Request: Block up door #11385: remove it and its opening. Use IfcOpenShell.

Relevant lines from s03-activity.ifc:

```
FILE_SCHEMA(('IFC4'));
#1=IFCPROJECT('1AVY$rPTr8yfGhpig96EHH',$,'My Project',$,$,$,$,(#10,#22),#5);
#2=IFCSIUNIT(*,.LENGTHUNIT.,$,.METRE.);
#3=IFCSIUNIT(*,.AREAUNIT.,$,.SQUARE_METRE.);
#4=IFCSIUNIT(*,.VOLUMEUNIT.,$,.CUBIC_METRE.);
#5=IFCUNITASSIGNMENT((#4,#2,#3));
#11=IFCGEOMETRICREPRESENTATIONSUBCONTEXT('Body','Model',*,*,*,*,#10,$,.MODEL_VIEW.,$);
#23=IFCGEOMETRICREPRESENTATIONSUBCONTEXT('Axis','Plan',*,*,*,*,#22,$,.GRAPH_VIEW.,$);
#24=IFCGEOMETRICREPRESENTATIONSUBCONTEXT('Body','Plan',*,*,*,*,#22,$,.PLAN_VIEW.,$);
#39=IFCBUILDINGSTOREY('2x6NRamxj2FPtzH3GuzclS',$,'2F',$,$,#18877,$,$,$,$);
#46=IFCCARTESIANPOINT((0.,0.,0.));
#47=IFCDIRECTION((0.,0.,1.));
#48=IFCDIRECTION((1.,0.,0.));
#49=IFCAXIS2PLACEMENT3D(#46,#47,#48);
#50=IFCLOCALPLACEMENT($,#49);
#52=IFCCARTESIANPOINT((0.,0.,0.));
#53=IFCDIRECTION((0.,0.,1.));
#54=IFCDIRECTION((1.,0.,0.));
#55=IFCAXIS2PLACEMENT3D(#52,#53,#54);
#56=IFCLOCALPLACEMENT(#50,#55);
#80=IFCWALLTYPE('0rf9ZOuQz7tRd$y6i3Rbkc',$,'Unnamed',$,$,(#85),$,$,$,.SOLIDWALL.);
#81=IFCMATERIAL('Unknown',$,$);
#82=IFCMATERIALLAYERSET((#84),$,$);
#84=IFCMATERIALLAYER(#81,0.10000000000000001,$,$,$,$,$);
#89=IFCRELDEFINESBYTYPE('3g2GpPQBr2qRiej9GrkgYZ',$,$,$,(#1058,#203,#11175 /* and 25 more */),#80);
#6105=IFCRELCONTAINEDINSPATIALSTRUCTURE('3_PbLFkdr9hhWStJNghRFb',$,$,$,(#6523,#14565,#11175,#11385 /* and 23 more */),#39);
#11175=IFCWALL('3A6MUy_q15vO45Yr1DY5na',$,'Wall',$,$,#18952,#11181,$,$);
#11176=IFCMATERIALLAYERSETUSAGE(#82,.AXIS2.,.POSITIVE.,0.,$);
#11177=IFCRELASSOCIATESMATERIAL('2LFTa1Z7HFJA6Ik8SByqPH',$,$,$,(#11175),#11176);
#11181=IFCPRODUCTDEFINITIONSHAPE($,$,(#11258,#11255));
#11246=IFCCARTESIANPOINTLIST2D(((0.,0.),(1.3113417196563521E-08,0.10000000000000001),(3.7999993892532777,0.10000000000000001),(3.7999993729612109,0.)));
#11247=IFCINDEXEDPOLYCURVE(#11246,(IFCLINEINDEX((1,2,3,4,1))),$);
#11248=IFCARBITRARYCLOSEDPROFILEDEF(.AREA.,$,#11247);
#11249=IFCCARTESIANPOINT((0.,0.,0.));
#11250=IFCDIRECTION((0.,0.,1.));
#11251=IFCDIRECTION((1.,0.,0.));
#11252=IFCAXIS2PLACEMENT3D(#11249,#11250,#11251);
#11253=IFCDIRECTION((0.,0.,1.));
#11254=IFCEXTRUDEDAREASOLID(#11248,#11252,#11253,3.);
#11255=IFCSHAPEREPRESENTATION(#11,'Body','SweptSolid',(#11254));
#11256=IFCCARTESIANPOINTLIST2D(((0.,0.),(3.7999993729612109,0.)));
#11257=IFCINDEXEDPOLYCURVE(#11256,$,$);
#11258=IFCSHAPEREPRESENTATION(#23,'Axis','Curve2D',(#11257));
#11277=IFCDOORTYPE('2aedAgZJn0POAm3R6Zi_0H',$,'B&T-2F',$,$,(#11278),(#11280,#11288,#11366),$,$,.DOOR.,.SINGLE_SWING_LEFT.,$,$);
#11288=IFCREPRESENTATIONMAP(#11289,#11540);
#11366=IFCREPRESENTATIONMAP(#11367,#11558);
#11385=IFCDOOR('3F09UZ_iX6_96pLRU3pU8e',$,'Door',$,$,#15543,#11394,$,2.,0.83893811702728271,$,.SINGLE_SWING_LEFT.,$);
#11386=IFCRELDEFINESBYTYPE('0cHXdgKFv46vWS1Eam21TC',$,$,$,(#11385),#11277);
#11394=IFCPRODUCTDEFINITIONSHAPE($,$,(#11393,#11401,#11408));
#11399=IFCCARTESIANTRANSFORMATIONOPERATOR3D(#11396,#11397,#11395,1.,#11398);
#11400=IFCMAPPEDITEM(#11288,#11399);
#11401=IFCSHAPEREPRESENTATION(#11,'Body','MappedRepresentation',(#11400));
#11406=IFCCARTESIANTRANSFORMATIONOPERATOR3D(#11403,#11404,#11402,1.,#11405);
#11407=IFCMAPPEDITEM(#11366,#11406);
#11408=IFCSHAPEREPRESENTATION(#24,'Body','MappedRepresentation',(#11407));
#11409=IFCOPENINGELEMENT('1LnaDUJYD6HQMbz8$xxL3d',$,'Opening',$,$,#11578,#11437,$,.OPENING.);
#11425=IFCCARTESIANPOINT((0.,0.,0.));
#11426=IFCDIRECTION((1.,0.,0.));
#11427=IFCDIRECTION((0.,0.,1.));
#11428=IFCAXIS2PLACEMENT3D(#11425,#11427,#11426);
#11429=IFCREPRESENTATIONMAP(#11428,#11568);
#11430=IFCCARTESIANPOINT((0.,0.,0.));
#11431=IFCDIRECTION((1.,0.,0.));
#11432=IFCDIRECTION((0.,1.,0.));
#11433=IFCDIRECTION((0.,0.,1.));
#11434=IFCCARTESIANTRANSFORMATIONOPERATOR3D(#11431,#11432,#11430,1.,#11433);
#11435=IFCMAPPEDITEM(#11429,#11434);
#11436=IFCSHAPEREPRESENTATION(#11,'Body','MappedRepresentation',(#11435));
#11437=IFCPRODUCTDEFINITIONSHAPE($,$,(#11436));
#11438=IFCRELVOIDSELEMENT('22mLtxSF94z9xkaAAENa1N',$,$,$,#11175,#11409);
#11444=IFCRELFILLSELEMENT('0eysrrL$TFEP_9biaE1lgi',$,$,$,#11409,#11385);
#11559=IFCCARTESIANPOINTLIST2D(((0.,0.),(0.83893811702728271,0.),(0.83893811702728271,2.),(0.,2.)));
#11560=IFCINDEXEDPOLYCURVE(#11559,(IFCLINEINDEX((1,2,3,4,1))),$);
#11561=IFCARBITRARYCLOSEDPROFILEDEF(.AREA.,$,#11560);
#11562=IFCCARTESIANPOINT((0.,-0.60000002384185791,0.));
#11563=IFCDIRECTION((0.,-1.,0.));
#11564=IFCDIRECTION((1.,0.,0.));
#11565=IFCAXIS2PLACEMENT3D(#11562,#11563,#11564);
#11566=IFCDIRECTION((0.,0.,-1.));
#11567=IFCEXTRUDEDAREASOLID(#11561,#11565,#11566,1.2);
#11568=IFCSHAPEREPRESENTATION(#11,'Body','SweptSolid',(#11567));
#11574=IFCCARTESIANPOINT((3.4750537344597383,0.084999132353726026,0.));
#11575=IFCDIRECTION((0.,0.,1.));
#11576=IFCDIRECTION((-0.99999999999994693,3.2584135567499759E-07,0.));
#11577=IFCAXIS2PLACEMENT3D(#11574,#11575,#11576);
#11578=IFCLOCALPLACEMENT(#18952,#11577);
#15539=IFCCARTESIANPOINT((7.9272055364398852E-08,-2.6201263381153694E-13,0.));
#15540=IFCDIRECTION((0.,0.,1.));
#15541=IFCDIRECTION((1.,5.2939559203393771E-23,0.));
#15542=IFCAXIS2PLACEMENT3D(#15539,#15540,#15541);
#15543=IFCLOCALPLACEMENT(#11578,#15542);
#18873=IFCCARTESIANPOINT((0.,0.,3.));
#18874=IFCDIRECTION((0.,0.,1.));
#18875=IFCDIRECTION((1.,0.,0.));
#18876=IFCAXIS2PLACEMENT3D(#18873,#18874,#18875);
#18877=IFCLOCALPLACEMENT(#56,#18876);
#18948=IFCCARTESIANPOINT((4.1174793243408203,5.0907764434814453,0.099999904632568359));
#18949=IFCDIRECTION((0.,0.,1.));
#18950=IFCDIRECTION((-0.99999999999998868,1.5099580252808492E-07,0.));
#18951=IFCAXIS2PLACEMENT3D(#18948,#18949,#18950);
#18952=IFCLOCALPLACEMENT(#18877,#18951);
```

```python
import ifcopenshell
import ifcopenshell.api.feature
import ifcopenshell.api.root
import ifcopenshell.geom
import ifcopenshell.util.shape

model = ifcopenshell.open("s03-activity.ifc")
settings = ifcopenshell.geom.settings()


def volume(element):
    """Net volume in cubic metres, openings subtracted."""
    shape = ifcopenshell.geom.create_shape(settings, element)
    return ifcopenshell.util.shape.get_volume(shape.geometry)


door = model.by_guid("3F09UZ_iX6_96pLRU3pU8e")
opening = door.FillsVoids[0].RelatingOpeningElement
wall = opening.VoidsElements[0].RelatingBuildingElement
before = volume(wall)

ifcopenshell.api.root.remove_product(model, product=door)
ifcopenshell.api.feature.remove_feature(model, feature=opening)

after = volume(wall)

print(f"wall volume {before:.3f} -> {after:.3f} m3")

model.write("s03-activity_rev.ifc")
```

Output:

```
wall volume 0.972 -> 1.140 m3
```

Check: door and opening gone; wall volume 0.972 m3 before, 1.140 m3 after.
